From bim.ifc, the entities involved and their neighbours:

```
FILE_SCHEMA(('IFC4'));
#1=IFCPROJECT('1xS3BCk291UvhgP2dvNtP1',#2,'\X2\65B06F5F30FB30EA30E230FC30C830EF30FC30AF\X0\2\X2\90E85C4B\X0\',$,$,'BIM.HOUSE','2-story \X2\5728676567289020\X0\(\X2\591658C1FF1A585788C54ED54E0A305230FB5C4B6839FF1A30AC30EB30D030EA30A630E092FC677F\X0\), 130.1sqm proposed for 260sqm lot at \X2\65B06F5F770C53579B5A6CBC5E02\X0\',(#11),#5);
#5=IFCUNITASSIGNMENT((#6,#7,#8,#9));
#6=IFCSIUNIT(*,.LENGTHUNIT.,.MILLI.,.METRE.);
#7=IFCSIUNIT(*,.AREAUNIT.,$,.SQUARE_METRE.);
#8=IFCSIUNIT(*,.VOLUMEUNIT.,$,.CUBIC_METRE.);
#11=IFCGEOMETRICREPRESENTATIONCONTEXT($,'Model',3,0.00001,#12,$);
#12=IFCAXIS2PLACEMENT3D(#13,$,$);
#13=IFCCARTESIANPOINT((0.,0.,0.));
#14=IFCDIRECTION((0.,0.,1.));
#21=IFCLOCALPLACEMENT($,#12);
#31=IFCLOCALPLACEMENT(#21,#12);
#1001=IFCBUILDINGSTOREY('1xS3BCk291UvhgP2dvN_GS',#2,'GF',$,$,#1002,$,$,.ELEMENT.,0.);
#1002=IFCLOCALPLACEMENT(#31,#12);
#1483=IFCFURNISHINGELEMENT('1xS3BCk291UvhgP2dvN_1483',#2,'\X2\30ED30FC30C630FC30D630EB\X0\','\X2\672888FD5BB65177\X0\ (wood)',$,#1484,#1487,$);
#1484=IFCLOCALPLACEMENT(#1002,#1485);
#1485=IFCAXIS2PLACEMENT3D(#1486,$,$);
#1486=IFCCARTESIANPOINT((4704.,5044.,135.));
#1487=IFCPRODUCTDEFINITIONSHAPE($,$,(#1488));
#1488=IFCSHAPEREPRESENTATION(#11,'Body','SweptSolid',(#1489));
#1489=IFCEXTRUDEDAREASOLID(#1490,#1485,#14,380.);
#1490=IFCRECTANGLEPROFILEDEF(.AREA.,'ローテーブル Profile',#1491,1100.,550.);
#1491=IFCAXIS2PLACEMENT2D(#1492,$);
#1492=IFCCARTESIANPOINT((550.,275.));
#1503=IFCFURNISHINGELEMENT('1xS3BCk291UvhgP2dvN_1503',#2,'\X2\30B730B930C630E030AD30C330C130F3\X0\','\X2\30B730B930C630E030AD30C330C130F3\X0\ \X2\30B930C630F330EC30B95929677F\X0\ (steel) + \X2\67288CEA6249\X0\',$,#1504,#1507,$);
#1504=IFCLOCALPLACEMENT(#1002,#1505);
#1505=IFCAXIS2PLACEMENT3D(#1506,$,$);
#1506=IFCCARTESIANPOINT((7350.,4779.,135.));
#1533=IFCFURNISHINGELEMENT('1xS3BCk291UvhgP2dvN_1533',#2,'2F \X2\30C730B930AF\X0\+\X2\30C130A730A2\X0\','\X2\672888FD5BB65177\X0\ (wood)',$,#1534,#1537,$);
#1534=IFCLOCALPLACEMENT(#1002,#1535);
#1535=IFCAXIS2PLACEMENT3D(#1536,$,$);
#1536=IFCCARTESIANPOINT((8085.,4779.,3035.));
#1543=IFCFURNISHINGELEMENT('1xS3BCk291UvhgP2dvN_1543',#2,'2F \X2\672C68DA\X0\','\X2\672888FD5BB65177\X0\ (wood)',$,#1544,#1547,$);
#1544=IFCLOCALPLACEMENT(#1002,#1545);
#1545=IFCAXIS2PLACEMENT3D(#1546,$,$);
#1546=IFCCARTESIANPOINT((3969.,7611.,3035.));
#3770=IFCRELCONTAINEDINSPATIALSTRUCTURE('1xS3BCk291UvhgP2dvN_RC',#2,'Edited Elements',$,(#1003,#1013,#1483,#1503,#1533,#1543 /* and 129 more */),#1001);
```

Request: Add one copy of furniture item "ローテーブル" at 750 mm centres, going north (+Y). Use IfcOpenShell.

```python
import numpy as np
import ifcopenshell
import ifcopenshell.api.geometry
import ifcopenshell.api.root
import ifcopenshell.util.element
import ifcopenshell.util.placement
import ifcopenshell.util.unit

model = ifcopenshell.open("bim.ifc")
unit_scale = ifcopenshell.util.unit.calculate_unit_scale(model)


def reuse_history(source, copy):
    """copy_class also copies each property set's owner history, people and application; keep the originals."""
    for rel in copy.IsDefinedBy:
        if rel.is_a("IfcRelDefinesByProperties") and (history := rel.RelatingPropertyDefinition.OwnerHistory):
            rel.RelatingPropertyDefinition.OwnerHistory = source.OwnerHistory
            ifcopenshell.util.element.remove_deep2(model, history)


source = model.by_guid("1xS3BCk291UvhgP2dvN_1483")
base = ifcopenshell.util.placement.get_local_placement(source.ObjectPlacement)
step = np.array([0.0, 1.0, 0.0]) * 0.75 / unit_scale

for i in range(1, 2):
    copy = ifcopenshell.api.root.copy_class(model, product=source)
    copy.Representation = ifcopenshell.util.element.copy_deep(
        model, source.Representation, exclude=["IfcGeometricRepresentationContext", "IfcRepresentationMap"]
    )
    reuse_history(source, copy)
    matrix = base.copy()
    matrix[:3, 3] += i * step
    print("added at", matrix[:3, 3].round(3) + 0.0)
    ifcopenshell.api.geometry.edit_object_placement(model, product=copy, matrix=matrix, is_si=False)

model.write("bim-out.ifc")
```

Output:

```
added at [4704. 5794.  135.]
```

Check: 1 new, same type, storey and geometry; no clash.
